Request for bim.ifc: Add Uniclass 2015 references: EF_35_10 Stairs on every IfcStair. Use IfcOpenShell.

First a look at what the model holds.

```python
import ifcopenshell

model = ifcopenshell.open("bim.ifc")
print(model.schema)
print("classifications:", [c.Name for c in model.by_type("IfcClassification")])
for ifc_class in ("IfcDoor", "IfcRoof", "IfcStair", "IfcWall", "IfcWindow"):
    print(ifc_class, len(model.by_type(ifc_class)))
```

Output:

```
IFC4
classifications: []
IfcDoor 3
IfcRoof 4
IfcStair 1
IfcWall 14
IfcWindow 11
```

```python
import ifcopenshell
import ifcopenshell.api.classification

model = ifcopenshell.open("bim.ifc")

system = ifcopenshell.api.classification.add_classification(model, classification="Uniclass 2015")

codes = {
    "IfcStair": ("EF_35_10", "Stairs"),
}
for ifc_class, (code, name) in codes.items():
    products = model.by_type(ifc_class)
    ifcopenshell.api.classification.add_reference(
        model, products=products, classification=system, identification=code, name=name
    )
    print(code, len(products))

model.write("bim_edited.ifc")
```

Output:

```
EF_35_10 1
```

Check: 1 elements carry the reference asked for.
